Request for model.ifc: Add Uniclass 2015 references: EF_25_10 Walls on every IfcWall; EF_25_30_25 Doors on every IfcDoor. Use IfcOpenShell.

First a look at what the model holds.

```python
import ifcopenshell

model = ifcopenshell.open("model.ifc")
print(model.schema)
print("classifications:", [c.Name for c in model.by_type("IfcClassification")])
for ifc_class in ("IfcDoor", "IfcRoof", "IfcStair", "IfcWall", "IfcWindow"):
    print(ifc_class, len(model.by_type(ifc_class)))
```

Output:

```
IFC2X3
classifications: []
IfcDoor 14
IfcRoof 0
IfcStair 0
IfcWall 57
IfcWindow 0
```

```python
import ifcopenshell
import ifcopenshell.api.classification

model = ifcopenshell.open("model.ifc")

# IFC2X3 requires Source and Edition and has no link from the project to the system.
system = model.create_entity("IfcClassification", Source="NBS", Edition="2015", Name="Uniclass 2015")

codes = {
    "IfcWall": ("EF_25_10", "Walls"),
    "IfcDoor": ("EF_25_30_25", "Doors"),
}
for ifc_class, (code, name) in codes.items():
    products = model.by_type(ifc_class)
    ifcopenshell.api.classification.add_reference(
        model, products=products, classification=system, identification=code, name=name
    )
    print(code, len(products))

model.write("model-out.ifc")
```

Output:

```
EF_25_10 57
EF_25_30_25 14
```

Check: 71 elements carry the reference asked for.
